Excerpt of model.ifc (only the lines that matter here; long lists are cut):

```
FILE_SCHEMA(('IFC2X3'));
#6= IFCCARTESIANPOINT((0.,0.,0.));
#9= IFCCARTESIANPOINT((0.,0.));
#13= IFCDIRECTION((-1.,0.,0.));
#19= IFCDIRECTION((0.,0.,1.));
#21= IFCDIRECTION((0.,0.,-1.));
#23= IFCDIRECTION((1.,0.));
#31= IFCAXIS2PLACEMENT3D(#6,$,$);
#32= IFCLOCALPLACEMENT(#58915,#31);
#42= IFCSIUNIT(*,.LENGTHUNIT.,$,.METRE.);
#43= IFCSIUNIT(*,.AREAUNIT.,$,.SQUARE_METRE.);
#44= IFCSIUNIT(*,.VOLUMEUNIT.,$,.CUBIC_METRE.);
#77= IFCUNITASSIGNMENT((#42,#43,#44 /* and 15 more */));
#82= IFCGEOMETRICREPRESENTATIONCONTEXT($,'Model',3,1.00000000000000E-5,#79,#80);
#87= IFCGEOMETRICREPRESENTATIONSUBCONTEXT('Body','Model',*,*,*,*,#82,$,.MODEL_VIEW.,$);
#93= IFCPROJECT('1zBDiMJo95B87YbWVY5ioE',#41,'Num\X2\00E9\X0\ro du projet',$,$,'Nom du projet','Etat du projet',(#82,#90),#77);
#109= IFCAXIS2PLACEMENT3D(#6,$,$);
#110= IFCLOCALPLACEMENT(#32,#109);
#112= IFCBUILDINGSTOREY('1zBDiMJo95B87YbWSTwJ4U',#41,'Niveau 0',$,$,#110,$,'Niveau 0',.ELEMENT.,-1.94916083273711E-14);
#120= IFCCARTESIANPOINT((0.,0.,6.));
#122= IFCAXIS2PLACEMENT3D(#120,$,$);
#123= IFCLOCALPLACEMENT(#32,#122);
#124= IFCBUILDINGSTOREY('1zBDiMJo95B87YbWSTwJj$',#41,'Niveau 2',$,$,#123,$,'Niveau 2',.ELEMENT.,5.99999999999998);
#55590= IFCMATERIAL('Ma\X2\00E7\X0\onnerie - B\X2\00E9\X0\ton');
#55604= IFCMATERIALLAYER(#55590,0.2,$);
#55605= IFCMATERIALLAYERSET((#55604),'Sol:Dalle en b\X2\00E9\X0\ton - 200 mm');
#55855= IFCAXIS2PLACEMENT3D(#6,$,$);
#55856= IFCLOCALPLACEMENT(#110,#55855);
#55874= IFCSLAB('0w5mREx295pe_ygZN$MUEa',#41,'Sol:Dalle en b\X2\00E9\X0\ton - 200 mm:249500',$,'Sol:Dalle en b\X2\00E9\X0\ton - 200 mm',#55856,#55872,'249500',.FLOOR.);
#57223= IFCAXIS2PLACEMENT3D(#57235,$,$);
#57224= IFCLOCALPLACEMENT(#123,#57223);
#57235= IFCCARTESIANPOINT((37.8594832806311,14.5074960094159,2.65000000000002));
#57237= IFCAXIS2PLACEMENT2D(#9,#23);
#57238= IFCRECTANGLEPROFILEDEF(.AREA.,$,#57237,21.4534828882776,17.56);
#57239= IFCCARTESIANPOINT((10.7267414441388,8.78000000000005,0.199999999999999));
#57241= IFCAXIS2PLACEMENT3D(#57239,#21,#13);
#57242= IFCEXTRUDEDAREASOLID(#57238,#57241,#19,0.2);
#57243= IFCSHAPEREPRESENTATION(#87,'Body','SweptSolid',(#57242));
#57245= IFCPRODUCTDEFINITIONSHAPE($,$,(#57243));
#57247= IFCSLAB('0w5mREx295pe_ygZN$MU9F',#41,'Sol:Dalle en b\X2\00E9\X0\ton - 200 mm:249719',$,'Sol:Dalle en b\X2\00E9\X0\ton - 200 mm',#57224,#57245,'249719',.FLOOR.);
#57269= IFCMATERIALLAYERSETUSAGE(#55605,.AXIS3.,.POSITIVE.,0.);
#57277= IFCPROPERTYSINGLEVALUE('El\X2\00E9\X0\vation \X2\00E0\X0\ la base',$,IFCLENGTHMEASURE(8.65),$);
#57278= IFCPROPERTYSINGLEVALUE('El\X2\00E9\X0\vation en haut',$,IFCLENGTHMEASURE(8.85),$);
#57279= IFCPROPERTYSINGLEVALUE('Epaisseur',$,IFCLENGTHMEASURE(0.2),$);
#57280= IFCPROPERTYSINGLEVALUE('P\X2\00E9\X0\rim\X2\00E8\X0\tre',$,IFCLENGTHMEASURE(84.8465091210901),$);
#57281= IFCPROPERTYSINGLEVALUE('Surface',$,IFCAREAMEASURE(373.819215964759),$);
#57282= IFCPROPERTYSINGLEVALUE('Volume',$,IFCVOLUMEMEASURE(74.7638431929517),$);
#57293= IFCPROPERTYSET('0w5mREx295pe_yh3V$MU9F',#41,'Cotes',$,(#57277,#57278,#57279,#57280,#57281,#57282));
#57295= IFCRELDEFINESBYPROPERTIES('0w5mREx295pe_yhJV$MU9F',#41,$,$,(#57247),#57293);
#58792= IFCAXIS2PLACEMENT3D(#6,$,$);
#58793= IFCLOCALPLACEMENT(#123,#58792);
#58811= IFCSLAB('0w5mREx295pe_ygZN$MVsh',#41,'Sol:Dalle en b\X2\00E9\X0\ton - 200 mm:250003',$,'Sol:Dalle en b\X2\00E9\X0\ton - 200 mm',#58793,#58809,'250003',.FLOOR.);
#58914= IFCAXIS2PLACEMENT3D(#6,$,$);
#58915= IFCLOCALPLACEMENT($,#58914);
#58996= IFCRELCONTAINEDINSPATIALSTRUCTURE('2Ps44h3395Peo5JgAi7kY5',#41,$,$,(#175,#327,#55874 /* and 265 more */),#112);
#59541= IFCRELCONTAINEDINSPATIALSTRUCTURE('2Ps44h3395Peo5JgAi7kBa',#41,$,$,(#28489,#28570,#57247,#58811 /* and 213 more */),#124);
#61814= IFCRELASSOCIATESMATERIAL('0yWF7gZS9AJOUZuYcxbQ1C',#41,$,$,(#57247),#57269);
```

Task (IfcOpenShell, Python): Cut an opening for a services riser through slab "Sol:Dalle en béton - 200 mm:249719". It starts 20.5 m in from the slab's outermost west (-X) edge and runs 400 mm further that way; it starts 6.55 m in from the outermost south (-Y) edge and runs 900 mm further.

```python
import numpy as np
import ifcopenshell
import ifcopenshell.api.feature
import ifcopenshell.api.geometry
import ifcopenshell.api.pset
import ifcopenshell.api.root
import ifcopenshell.geom
import ifcopenshell.util.element
import ifcopenshell.util.placement
import ifcopenshell.util.representation
import ifcopenshell.util.shape
import ifcopenshell.util.unit

model = ifcopenshell.open("model.ifc")
unit_scale = ifcopenshell.util.unit.calculate_unit_scale(model)
area_scale = ifcopenshell.util.unit.calculate_unit_scale(model, "AREAUNIT")
volume_scale = ifcopenshell.util.unit.calculate_unit_scale(model, "VOLUMEUNIT")
settings = ifcopenshell.geom.settings()


def volume(element):
    """Net volume in cubic metres, openings subtracted."""
    shape = ifcopenshell.geom.create_shape(settings, element)
    return ifcopenshell.util.shape.get_volume(shape.geometry)


slab = model.by_id(57247)
before = volume(slab)

# Extent in the slab's own axes, in metres. The edges named are its -X and -Y sides.
slab_shape = ifcopenshell.geom.create_shape(settings, slab)
vertices = ifcopenshell.util.shape.get_vertices(slab_shape.geometry)
x_min, y_min, bottom = vertices.min(axis=0)
top = vertices[:, 2].max()

opening = ifcopenshell.api.root.create_entity(model, ifc_class="IfcOpeningElement", name="Services riser opening")
context = ifcopenshell.util.representation.get_context(model, "Model", "Body", "MODEL_VIEW")
width, depth = 0.4, 0.9
outline = [(0.0, 0.0), (width, 0.0), (width, depth), (0.0, depth), (0.0, 0.0)]
# Overshoot both faces by 50 mm so the cut is clean.
shape = ifcopenshell.api.geometry.add_slab_representation(
    model, context=context, depth=top - bottom + 0.1, polyline=outline
)
ifcopenshell.api.geometry.assign_representation(model, product=opening, representation=shape)

matrix = ifcopenshell.util.placement.get_local_placement(slab.ObjectPlacement)
matrix[:, 3] = matrix @ np.append(np.array([x_min + 20.5, y_min + 6.55, bottom - 0.05]) / unit_scale, 1.0)
ifcopenshell.api.geometry.edit_object_placement(model, product=opening, matrix=matrix, is_si=False)
ifcopenshell.api.feature.add_feature(model, feature=opening, element=slab)

after = volume(slab)

# Update the slab's stored quantities.
pset = model.by_id(ifcopenshell.util.element.get_pset(slab, "Cotes", should_inherit=False)["id"])
ifcopenshell.api.pset.edit_pset(model, pset=pset, properties={
    "Surface": model.create_entity("IfcAreaMeasure", after / (top - bottom) / area_scale),
    "Volume": model.create_entity("IfcVolumeMeasure", after / volume_scale),
})

print(f"slab volume {before:.3f} -> {after:.3f} m3")

model.write("model_v2.ifc")
```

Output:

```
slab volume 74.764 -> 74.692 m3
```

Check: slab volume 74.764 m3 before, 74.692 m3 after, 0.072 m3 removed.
